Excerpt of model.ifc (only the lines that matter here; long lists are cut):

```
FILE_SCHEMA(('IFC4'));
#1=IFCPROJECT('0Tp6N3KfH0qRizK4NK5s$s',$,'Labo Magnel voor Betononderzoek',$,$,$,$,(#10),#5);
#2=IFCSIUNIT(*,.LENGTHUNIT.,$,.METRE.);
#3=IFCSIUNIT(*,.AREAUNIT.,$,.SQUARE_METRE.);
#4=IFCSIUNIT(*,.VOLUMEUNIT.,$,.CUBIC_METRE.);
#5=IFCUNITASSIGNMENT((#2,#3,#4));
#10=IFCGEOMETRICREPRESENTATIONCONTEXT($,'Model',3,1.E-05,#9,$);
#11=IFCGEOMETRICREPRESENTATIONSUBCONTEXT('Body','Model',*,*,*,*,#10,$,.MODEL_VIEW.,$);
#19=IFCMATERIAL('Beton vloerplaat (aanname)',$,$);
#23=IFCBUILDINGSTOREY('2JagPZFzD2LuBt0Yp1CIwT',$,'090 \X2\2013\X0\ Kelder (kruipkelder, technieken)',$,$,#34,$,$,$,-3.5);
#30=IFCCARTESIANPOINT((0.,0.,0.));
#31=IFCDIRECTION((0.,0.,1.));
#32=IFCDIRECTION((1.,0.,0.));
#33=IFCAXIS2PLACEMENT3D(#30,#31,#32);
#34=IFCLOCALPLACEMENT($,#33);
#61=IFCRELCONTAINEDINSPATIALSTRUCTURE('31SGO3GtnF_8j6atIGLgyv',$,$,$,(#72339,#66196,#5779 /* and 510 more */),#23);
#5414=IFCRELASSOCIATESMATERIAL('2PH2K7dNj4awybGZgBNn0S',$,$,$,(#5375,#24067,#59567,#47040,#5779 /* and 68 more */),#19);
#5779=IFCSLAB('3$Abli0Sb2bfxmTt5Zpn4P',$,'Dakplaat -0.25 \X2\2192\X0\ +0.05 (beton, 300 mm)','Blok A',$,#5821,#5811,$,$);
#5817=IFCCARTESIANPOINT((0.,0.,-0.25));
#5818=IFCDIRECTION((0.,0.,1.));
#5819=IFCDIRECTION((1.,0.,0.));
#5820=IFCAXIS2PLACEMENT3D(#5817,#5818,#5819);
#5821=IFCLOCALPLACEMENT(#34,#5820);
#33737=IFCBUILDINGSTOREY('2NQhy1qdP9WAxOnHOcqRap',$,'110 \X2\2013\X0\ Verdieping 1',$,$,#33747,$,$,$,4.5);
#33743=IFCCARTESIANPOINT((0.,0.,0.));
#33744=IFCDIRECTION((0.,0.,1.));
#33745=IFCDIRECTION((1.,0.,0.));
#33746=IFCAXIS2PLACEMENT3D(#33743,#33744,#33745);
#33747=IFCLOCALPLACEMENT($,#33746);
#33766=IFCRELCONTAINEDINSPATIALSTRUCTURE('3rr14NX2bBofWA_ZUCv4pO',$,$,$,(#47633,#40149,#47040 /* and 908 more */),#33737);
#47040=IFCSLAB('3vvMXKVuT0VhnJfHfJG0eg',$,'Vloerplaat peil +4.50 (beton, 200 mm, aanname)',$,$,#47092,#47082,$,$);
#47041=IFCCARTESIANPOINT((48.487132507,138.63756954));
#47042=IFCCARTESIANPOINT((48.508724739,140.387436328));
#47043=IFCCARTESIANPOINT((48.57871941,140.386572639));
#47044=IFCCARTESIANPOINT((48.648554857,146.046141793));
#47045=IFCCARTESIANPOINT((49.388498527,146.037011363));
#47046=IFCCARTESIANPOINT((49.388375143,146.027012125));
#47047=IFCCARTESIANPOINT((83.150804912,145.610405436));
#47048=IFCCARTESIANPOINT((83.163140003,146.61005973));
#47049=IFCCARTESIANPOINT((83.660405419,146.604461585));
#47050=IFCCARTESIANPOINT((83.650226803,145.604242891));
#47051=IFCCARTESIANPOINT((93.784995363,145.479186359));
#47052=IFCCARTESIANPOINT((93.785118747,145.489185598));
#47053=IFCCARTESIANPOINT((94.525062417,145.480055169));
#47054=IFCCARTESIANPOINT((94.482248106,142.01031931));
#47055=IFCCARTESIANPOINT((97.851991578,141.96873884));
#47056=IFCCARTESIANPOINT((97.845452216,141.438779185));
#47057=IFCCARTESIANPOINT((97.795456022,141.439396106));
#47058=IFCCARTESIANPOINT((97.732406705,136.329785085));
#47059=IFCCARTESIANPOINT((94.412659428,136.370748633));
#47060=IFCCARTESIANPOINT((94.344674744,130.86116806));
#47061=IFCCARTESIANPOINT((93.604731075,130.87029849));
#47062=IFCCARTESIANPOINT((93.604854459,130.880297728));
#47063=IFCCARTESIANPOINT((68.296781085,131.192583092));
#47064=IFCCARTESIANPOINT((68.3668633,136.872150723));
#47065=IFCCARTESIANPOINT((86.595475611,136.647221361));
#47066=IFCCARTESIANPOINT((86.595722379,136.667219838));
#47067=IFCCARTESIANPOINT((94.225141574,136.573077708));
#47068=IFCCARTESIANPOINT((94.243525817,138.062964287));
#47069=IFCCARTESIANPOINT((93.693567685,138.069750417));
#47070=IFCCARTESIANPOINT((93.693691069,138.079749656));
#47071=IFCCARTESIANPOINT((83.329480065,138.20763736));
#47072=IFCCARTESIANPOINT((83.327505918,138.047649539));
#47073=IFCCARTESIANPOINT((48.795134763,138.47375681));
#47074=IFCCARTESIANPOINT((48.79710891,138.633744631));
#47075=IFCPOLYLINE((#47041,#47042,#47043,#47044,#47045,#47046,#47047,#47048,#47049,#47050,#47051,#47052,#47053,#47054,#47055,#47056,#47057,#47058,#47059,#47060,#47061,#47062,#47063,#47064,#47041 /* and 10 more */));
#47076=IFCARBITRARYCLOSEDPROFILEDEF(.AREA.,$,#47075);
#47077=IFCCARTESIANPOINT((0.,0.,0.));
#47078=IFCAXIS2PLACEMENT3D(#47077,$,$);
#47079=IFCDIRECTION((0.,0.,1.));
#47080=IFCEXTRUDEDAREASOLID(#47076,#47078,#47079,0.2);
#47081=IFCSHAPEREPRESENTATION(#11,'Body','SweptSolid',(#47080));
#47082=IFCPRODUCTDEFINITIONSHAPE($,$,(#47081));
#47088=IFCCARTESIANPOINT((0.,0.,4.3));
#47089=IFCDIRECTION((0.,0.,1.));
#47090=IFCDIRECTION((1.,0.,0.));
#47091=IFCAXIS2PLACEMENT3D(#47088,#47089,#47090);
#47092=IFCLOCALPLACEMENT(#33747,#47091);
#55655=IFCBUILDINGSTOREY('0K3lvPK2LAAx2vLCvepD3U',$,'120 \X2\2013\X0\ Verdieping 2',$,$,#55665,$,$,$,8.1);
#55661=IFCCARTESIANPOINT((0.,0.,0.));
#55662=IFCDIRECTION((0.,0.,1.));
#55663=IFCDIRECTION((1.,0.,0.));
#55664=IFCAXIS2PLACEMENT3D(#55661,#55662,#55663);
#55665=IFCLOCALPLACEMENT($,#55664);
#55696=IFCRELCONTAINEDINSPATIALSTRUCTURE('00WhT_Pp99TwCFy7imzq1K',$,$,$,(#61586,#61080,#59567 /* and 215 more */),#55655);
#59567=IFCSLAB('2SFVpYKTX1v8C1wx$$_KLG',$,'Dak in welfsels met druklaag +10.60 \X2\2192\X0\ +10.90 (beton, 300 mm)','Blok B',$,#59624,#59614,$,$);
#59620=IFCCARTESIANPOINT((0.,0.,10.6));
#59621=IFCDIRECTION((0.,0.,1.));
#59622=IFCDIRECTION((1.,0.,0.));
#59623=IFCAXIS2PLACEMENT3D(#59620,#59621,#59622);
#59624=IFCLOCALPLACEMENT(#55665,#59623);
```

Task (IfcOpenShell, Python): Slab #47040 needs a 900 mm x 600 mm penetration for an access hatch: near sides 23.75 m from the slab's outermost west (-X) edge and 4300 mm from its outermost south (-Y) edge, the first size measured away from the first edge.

```python
import numpy as np
import ifcopenshell
import ifcopenshell.api.feature
import ifcopenshell.api.geometry
import ifcopenshell.api.root
import ifcopenshell.geom
import ifcopenshell.util.placement
import ifcopenshell.util.representation
import ifcopenshell.util.shape
import ifcopenshell.util.unit

model = ifcopenshell.open("model.ifc")
unit_scale = ifcopenshell.util.unit.calculate_unit_scale(model)
settings = ifcopenshell.geom.settings()


def volume(element):
    """Net volume in cubic metres, openings subtracted."""
    shape = ifcopenshell.geom.create_shape(settings, element)
    return ifcopenshell.util.shape.get_volume(shape.geometry)


slab = model.by_id(47040)
before = volume(slab)

# Extent in the slab's own axes, in metres. The edges named are its -X and -Y sides.
slab_shape = ifcopenshell.geom.create_shape(settings, slab)
vertices = ifcopenshell.util.shape.get_vertices(slab_shape.geometry)
x_min, y_min, bottom = vertices.min(axis=0)
top = vertices[:, 2].max()

opening = ifcopenshell.api.root.create_entity(model, ifc_class="IfcOpeningElement", name="Access hatch opening", predefined_type="OPENING")
context = ifcopenshell.util.representation.get_context(model, "Model", "Body", "MODEL_VIEW")
width, depth = 0.9, 0.6
outline = [(0.0, 0.0), (width, 0.0), (width, depth), (0.0, depth), (0.0, 0.0)]
# Overshoot both faces by 50 mm so the cut is clean.
shape = ifcopenshell.api.geometry.add_slab_representation(
    model, context=context, depth=top - bottom + 0.1, polyline=outline
)
ifcopenshell.api.geometry.assign_representation(model, product=opening, representation=shape)

matrix = ifcopenshell.util.placement.get_local_placement(slab.ObjectPlacement)
matrix[:, 3] = matrix @ np.append(np.array([x_min + 23.75, y_min + 4.3, bottom - 0.05]) / unit_scale, 1.0)
ifcopenshell.api.geometry.edit_object_placement(model, product=opening, matrix=matrix, is_si=False)
ifcopenshell.api.feature.add_feature(model, feature=opening, element=slab)

after = volume(slab)

print(f"slab volume {before:.3f} -> {after:.3f} m3")

model.write("model_edited.ifc")
```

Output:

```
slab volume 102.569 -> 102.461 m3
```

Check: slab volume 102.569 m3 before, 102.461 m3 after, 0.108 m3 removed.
